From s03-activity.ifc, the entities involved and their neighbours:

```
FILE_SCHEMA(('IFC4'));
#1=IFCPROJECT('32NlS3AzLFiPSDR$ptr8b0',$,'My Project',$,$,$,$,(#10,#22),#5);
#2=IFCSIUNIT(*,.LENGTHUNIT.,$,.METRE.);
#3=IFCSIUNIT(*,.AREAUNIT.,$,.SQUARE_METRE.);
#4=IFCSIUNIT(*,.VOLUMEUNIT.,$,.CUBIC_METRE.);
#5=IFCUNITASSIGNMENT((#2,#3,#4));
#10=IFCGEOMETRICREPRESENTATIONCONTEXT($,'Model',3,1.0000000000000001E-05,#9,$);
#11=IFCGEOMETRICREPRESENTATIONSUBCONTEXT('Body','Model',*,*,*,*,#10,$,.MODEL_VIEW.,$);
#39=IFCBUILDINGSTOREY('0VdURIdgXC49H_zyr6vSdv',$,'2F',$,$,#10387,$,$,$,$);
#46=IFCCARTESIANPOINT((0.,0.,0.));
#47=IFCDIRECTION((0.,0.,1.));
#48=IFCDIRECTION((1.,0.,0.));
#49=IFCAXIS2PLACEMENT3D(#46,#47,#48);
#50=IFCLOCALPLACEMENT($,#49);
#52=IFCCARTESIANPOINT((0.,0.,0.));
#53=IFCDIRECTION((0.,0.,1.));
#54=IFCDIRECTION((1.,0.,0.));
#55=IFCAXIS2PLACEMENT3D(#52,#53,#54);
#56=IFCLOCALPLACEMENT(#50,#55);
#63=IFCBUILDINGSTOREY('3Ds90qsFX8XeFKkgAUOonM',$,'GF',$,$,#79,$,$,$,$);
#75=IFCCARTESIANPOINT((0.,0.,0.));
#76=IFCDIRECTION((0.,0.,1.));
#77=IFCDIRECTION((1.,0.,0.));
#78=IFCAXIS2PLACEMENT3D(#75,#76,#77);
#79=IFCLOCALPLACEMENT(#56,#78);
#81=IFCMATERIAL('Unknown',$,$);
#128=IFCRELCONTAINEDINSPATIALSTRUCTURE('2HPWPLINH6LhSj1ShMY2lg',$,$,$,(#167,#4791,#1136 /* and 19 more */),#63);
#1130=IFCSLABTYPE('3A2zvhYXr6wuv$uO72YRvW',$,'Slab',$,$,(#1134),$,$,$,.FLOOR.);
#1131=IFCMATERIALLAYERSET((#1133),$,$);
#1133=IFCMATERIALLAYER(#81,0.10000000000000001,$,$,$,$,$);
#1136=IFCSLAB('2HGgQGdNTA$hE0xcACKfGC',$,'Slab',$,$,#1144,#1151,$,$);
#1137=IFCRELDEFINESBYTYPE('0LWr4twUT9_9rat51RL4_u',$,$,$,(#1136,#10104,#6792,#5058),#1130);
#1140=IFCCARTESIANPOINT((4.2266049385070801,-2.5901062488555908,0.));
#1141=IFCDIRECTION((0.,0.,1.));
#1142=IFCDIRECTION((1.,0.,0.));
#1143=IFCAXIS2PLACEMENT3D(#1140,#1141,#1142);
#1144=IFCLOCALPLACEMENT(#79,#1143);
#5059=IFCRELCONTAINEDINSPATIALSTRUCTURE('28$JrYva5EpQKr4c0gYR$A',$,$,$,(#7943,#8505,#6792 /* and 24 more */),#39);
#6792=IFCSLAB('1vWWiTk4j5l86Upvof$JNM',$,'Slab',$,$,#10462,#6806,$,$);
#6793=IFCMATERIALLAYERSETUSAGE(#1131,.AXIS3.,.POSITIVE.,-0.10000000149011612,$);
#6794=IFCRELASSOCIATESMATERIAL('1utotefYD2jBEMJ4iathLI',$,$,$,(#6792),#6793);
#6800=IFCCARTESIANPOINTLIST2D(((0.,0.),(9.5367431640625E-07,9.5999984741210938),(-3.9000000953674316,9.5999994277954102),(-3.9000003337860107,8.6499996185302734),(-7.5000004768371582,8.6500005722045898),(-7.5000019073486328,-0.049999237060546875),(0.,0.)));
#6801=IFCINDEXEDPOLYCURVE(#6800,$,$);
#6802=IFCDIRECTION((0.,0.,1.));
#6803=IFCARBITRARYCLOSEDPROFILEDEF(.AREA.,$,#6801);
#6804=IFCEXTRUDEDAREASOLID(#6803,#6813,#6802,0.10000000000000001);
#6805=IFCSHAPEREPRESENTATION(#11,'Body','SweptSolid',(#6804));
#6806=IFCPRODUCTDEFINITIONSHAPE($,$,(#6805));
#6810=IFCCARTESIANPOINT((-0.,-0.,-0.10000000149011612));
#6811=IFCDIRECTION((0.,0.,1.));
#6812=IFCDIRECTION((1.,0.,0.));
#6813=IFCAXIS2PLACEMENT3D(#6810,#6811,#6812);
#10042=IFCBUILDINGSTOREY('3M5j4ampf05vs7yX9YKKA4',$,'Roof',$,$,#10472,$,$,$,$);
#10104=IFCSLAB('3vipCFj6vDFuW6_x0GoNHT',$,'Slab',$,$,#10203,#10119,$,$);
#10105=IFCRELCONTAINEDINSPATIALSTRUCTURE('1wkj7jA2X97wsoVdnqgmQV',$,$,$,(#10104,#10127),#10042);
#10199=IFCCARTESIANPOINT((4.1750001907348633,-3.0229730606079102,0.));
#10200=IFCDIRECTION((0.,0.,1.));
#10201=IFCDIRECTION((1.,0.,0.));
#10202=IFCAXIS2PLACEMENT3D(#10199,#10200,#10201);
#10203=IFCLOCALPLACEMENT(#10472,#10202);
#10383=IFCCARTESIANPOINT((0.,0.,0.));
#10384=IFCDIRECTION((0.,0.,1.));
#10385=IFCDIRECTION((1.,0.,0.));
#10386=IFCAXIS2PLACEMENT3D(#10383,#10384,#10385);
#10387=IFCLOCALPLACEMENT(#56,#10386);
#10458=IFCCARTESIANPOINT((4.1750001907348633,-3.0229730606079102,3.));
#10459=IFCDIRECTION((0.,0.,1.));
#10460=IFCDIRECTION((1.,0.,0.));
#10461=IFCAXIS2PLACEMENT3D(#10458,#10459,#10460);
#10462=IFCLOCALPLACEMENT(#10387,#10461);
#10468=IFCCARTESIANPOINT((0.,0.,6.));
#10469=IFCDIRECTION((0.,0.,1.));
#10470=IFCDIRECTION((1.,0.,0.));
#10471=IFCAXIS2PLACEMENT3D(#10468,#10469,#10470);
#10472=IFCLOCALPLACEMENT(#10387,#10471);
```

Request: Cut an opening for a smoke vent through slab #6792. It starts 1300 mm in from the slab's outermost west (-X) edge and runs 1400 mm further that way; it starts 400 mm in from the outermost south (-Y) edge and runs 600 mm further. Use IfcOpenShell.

```python
import numpy as np
import ifcopenshell
import ifcopenshell.api.feature
import ifcopenshell.api.geometry
import ifcopenshell.api.root
import ifcopenshell.geom
import ifcopenshell.util.placement
import ifcopenshell.util.representation
import ifcopenshell.util.shape
import ifcopenshell.util.unit

model = ifcopenshell.open("s03-activity.ifc")
unit_scale = ifcopenshell.util.unit.calculate_unit_scale(model)
settings = ifcopenshell.geom.settings()


def volume(element):
    """Net volume in cubic metres, openings subtracted."""
    shape = ifcopenshell.geom.create_shape(settings, element)
    return ifcopenshell.util.shape.get_volume(shape.geometry)


slab = model.by_guid("1vWWiTk4j5l86Upvof$JNM")
before = volume(slab)

# Extent in the slab's own axes, in metres. The edges named are its -X and -Y sides.
slab_shape = ifcopenshell.geom.create_shape(settings, slab)
vertices = ifcopenshell.util.shape.get_vertices(slab_shape.geometry)
x_min, y_min, bottom = vertices.min(axis=0)
top = vertices[:, 2].max()

opening = ifcopenshell.api.root.create_entity(model, ifc_class="IfcOpeningElement", name="Smoke vent opening", predefined_type="OPENING")
context = ifcopenshell.util.representation.get_context(model, "Model", "Body", "MODEL_VIEW")
width, depth = 1.4, 0.6
outline = [(0.0, 0.0), (width, 0.0), (width, depth), (0.0, depth), (0.0, 0.0)]
# Overshoot both faces by 50 mm so the cut is clean.
shape = ifcopenshell.api.geometry.add_slab_representation(
    model, context=context, depth=top - bottom + 0.1, polyline=outline
)
ifcopenshell.api.geometry.assign_representation(model, product=opening, representation=shape)

matrix = ifcopenshell.util.placement.get_local_placement(slab.ObjectPlacement)
matrix[:, 3] = matrix @ np.append(np.array([x_min + 1.3, y_min + 0.4, bottom - 0.05]) / unit_scale, 1.0)
ifcopenshell.api.geometry.edit_object_placement(model, product=opening, matrix=matrix, is_si=False)
ifcopenshell.api.feature.add_feature(model, feature=opening, element=slab)

after = volume(slab)

print(f"slab volume {before:.3f} -> {after:.3f} m3")

model.write("s03-activity_rev.ifc")
```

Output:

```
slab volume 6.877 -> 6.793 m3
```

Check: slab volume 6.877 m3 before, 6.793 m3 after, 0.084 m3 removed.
